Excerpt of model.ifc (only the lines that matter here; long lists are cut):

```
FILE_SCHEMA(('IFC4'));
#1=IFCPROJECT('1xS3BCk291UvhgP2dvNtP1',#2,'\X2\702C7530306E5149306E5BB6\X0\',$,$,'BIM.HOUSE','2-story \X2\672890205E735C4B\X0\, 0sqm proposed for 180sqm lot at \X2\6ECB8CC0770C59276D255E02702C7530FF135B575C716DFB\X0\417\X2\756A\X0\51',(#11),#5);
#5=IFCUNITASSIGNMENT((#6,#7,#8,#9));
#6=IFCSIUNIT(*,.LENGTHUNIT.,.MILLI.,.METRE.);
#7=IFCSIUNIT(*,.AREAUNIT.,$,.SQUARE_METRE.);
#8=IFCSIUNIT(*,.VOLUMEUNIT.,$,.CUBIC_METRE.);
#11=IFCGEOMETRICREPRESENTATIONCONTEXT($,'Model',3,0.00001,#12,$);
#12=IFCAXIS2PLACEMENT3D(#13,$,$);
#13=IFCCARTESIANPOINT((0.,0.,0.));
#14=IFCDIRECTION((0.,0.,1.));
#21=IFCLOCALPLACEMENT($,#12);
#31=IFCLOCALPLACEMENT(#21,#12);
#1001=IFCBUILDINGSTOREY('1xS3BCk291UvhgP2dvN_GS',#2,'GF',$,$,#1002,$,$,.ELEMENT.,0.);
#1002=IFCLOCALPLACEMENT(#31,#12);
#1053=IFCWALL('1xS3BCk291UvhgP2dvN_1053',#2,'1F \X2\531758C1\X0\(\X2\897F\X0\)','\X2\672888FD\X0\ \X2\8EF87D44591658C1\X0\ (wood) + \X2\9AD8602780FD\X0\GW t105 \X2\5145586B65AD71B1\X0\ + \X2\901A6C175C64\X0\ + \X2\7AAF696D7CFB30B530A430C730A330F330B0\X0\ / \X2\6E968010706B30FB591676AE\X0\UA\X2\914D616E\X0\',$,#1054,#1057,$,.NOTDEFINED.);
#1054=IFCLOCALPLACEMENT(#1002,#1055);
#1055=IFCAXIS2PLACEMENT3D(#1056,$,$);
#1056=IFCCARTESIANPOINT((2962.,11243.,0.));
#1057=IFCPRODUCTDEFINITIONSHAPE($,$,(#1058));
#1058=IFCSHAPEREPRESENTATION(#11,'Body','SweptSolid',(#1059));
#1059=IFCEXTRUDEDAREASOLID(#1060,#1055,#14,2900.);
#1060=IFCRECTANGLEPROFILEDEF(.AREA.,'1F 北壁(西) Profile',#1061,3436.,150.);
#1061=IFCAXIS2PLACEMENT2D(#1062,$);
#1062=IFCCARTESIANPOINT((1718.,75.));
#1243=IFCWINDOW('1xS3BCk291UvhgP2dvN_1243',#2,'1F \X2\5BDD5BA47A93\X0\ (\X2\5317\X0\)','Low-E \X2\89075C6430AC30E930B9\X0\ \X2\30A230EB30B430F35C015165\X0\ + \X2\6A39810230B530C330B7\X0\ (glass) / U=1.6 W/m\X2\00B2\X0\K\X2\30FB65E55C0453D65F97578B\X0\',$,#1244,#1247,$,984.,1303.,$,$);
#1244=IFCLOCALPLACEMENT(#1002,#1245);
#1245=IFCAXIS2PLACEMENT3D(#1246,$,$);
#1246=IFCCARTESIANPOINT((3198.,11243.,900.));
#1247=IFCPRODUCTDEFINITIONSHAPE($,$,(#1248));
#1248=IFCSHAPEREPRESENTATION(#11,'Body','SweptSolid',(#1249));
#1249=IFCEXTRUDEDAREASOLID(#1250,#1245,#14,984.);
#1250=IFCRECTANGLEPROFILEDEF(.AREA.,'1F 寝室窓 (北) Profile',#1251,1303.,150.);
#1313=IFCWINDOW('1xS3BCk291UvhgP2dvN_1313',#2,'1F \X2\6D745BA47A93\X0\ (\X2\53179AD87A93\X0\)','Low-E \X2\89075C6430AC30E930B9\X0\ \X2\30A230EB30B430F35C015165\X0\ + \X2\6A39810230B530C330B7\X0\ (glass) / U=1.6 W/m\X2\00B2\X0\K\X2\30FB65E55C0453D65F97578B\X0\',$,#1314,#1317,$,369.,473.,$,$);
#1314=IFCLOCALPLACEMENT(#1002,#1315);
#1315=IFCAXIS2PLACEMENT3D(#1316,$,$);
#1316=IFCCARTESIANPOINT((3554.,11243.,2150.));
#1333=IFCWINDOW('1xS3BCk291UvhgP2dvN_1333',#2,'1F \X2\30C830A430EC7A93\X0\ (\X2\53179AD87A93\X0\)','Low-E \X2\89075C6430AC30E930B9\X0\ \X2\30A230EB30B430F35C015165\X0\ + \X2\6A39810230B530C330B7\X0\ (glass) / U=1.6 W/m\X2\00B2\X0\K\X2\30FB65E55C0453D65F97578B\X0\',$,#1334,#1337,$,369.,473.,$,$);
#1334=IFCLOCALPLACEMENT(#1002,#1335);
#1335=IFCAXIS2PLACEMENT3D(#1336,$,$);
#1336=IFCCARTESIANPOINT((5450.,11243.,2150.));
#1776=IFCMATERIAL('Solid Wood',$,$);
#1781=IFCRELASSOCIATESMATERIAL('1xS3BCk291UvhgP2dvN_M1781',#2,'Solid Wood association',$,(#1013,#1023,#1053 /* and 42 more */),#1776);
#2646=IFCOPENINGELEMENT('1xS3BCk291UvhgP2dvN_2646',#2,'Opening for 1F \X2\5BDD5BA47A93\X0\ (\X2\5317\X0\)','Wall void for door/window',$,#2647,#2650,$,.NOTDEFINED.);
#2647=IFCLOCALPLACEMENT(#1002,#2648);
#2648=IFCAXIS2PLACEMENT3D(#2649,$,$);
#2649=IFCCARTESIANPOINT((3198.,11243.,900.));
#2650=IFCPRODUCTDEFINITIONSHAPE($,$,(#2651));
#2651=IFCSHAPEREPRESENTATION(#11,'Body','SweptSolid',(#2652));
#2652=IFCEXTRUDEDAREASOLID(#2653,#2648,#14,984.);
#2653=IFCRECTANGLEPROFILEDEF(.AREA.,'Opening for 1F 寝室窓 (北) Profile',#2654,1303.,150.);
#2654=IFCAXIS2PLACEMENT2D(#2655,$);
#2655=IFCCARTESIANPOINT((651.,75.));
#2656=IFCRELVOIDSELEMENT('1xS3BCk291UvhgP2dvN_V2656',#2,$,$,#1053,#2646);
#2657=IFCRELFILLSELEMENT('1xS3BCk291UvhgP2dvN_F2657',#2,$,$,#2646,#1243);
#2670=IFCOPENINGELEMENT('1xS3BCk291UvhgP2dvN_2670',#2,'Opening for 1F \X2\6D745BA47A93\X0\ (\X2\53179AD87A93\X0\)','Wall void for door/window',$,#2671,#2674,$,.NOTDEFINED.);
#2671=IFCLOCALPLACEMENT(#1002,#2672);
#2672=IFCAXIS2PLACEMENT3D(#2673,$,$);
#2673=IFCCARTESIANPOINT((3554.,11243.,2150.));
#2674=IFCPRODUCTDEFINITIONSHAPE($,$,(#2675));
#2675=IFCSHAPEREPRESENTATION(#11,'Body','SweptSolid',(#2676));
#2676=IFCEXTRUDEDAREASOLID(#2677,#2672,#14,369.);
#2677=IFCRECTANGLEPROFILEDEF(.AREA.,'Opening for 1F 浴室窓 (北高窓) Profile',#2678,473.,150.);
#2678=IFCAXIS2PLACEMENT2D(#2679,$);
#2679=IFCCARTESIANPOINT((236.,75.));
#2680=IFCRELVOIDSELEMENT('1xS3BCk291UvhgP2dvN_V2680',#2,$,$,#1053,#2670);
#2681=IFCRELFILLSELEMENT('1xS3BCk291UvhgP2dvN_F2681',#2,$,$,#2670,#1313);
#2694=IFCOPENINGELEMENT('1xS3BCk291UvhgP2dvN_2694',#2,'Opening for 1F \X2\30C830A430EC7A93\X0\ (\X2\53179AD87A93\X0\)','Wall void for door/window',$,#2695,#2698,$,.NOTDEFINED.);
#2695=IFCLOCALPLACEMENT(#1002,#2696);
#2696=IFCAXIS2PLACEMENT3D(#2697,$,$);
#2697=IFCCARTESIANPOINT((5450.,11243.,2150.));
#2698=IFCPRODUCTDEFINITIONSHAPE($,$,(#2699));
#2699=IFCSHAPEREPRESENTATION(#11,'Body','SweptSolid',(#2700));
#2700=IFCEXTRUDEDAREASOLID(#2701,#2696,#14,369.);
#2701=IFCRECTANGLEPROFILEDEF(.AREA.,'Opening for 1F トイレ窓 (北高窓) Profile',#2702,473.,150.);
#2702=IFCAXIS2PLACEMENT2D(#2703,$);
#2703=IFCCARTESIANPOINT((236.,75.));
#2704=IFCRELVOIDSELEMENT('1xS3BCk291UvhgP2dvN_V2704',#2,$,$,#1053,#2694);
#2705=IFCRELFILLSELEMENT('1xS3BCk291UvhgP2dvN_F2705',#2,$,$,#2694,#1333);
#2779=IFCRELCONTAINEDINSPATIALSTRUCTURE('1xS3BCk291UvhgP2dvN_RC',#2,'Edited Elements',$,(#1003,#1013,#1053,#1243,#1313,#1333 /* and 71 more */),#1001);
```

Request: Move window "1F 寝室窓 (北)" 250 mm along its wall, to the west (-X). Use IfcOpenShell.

```python
import ifcopenshell
import ifcopenshell.api.geometry
import ifcopenshell.util.placement

model = ifcopenshell.open("model.ifc")

window = model.by_guid("1xS3BCk291UvhgP2dvN_1243")
opening = window.FillsVoids[0].RelatingOpeningElement
wall = opening.VoidsElements[0].RelatingBuildingElement

wall_matrix = ifcopenshell.util.placement.get_local_placement(wall.ObjectPlacement)
shift = wall_matrix[:3, 0] * -250.0
before = ifcopenshell.util.placement.get_local_placement(window.ObjectPlacement)[:3, 3].copy()

# The window is not placed relative to its opening, so move both.
for product in (opening, window):
    matrix = ifcopenshell.util.placement.get_local_placement(product.ObjectPlacement)
    matrix[:3, 3] += shift
    ifcopenshell.api.geometry.edit_object_placement(model, product=product, matrix=matrix, is_si=False)

after = ifcopenshell.util.placement.get_local_placement(window.ObjectPlacement)[:3, 3]
print("window moved by", (after - before).round(3) + 0.0)

model.write("model_v2.ifc")
```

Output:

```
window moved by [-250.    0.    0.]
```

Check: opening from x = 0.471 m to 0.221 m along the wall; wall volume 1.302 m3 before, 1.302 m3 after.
